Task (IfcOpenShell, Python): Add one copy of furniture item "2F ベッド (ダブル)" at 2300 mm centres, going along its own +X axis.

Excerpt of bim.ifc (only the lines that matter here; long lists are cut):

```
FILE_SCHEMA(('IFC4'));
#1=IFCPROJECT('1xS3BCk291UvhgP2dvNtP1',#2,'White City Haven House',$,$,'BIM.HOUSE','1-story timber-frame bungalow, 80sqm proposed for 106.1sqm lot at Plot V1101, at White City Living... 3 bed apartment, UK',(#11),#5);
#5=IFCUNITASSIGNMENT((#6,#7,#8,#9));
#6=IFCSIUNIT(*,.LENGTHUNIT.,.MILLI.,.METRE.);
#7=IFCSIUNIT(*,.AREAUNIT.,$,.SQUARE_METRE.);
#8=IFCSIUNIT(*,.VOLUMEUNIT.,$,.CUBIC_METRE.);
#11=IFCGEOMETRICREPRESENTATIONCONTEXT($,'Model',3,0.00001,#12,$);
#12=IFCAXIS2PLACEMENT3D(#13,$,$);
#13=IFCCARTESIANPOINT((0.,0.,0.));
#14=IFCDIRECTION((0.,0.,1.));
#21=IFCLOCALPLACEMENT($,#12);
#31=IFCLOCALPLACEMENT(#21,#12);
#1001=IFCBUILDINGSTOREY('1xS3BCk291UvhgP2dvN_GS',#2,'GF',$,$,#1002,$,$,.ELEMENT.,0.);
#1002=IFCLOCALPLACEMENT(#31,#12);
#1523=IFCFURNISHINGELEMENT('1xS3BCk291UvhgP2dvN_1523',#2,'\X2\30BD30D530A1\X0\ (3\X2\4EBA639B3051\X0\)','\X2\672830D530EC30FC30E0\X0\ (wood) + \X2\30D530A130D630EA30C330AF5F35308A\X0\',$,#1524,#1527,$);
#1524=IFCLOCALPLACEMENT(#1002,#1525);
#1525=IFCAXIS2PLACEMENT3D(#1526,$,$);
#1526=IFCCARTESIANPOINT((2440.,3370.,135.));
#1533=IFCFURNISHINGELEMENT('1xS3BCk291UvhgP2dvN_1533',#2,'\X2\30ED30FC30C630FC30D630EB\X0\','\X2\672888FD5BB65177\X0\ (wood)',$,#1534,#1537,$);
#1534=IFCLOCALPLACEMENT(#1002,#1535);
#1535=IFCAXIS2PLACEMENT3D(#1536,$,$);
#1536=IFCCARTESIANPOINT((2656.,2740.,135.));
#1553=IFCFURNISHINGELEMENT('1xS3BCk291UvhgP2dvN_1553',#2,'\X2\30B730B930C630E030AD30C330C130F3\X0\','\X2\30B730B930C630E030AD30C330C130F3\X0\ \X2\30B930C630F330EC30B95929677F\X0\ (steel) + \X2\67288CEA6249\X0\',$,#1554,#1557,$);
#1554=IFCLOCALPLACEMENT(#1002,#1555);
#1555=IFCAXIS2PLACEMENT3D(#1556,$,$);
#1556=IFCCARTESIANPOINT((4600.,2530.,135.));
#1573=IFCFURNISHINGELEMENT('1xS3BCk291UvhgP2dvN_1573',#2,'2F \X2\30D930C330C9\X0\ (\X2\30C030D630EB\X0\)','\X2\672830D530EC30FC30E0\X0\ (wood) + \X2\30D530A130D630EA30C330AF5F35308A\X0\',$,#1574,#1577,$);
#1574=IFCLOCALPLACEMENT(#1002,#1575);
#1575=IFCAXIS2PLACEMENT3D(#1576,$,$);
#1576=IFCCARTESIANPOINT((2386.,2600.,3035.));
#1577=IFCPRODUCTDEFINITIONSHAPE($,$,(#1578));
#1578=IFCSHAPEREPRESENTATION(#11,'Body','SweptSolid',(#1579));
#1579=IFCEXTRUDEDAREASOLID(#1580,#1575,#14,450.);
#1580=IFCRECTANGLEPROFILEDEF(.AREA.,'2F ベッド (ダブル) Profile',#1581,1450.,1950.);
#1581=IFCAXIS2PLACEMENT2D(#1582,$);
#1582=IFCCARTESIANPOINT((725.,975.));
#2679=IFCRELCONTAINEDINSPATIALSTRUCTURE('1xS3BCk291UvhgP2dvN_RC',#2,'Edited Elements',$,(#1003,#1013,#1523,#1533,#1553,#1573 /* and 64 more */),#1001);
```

```python
import ifcopenshell
import ifcopenshell.api.geometry
import ifcopenshell.api.root
import ifcopenshell.util.element
import ifcopenshell.util.placement

model = ifcopenshell.open("bim.ifc")


def reuse_history(source, copy):
    """copy_class also copies each property set's owner history, people and application; keep the originals."""
    for rel in copy.IsDefinedBy:
        if rel.is_a("IfcRelDefinesByProperties") and (history := rel.RelatingPropertyDefinition.OwnerHistory):
            rel.RelatingPropertyDefinition.OwnerHistory = source.OwnerHistory
            ifcopenshell.util.element.remove_deep2(model, history)


source = model.by_id(1573)
base = ifcopenshell.util.placement.get_local_placement(source.ObjectPlacement)
step = base[:3, 0] * 2300.0

for i in range(1, 2):
    copy = ifcopenshell.api.root.copy_class(model, product=source)
    copy.Representation = ifcopenshell.util.element.copy_deep(
        model, source.Representation, exclude=["IfcGeometricRepresentationContext", "IfcRepresentationMap"]
    )
    reuse_history(source, copy)
    matrix = base.copy()
    matrix[:3, 3] += i * step
    print("added at", matrix[:3, 3].round(3) + 0.0)
    ifcopenshell.api.geometry.edit_object_placement(model, product=copy, matrix=matrix, is_si=False)

model.write("bim-out.ifc")
```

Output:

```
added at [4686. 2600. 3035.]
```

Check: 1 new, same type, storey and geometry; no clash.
